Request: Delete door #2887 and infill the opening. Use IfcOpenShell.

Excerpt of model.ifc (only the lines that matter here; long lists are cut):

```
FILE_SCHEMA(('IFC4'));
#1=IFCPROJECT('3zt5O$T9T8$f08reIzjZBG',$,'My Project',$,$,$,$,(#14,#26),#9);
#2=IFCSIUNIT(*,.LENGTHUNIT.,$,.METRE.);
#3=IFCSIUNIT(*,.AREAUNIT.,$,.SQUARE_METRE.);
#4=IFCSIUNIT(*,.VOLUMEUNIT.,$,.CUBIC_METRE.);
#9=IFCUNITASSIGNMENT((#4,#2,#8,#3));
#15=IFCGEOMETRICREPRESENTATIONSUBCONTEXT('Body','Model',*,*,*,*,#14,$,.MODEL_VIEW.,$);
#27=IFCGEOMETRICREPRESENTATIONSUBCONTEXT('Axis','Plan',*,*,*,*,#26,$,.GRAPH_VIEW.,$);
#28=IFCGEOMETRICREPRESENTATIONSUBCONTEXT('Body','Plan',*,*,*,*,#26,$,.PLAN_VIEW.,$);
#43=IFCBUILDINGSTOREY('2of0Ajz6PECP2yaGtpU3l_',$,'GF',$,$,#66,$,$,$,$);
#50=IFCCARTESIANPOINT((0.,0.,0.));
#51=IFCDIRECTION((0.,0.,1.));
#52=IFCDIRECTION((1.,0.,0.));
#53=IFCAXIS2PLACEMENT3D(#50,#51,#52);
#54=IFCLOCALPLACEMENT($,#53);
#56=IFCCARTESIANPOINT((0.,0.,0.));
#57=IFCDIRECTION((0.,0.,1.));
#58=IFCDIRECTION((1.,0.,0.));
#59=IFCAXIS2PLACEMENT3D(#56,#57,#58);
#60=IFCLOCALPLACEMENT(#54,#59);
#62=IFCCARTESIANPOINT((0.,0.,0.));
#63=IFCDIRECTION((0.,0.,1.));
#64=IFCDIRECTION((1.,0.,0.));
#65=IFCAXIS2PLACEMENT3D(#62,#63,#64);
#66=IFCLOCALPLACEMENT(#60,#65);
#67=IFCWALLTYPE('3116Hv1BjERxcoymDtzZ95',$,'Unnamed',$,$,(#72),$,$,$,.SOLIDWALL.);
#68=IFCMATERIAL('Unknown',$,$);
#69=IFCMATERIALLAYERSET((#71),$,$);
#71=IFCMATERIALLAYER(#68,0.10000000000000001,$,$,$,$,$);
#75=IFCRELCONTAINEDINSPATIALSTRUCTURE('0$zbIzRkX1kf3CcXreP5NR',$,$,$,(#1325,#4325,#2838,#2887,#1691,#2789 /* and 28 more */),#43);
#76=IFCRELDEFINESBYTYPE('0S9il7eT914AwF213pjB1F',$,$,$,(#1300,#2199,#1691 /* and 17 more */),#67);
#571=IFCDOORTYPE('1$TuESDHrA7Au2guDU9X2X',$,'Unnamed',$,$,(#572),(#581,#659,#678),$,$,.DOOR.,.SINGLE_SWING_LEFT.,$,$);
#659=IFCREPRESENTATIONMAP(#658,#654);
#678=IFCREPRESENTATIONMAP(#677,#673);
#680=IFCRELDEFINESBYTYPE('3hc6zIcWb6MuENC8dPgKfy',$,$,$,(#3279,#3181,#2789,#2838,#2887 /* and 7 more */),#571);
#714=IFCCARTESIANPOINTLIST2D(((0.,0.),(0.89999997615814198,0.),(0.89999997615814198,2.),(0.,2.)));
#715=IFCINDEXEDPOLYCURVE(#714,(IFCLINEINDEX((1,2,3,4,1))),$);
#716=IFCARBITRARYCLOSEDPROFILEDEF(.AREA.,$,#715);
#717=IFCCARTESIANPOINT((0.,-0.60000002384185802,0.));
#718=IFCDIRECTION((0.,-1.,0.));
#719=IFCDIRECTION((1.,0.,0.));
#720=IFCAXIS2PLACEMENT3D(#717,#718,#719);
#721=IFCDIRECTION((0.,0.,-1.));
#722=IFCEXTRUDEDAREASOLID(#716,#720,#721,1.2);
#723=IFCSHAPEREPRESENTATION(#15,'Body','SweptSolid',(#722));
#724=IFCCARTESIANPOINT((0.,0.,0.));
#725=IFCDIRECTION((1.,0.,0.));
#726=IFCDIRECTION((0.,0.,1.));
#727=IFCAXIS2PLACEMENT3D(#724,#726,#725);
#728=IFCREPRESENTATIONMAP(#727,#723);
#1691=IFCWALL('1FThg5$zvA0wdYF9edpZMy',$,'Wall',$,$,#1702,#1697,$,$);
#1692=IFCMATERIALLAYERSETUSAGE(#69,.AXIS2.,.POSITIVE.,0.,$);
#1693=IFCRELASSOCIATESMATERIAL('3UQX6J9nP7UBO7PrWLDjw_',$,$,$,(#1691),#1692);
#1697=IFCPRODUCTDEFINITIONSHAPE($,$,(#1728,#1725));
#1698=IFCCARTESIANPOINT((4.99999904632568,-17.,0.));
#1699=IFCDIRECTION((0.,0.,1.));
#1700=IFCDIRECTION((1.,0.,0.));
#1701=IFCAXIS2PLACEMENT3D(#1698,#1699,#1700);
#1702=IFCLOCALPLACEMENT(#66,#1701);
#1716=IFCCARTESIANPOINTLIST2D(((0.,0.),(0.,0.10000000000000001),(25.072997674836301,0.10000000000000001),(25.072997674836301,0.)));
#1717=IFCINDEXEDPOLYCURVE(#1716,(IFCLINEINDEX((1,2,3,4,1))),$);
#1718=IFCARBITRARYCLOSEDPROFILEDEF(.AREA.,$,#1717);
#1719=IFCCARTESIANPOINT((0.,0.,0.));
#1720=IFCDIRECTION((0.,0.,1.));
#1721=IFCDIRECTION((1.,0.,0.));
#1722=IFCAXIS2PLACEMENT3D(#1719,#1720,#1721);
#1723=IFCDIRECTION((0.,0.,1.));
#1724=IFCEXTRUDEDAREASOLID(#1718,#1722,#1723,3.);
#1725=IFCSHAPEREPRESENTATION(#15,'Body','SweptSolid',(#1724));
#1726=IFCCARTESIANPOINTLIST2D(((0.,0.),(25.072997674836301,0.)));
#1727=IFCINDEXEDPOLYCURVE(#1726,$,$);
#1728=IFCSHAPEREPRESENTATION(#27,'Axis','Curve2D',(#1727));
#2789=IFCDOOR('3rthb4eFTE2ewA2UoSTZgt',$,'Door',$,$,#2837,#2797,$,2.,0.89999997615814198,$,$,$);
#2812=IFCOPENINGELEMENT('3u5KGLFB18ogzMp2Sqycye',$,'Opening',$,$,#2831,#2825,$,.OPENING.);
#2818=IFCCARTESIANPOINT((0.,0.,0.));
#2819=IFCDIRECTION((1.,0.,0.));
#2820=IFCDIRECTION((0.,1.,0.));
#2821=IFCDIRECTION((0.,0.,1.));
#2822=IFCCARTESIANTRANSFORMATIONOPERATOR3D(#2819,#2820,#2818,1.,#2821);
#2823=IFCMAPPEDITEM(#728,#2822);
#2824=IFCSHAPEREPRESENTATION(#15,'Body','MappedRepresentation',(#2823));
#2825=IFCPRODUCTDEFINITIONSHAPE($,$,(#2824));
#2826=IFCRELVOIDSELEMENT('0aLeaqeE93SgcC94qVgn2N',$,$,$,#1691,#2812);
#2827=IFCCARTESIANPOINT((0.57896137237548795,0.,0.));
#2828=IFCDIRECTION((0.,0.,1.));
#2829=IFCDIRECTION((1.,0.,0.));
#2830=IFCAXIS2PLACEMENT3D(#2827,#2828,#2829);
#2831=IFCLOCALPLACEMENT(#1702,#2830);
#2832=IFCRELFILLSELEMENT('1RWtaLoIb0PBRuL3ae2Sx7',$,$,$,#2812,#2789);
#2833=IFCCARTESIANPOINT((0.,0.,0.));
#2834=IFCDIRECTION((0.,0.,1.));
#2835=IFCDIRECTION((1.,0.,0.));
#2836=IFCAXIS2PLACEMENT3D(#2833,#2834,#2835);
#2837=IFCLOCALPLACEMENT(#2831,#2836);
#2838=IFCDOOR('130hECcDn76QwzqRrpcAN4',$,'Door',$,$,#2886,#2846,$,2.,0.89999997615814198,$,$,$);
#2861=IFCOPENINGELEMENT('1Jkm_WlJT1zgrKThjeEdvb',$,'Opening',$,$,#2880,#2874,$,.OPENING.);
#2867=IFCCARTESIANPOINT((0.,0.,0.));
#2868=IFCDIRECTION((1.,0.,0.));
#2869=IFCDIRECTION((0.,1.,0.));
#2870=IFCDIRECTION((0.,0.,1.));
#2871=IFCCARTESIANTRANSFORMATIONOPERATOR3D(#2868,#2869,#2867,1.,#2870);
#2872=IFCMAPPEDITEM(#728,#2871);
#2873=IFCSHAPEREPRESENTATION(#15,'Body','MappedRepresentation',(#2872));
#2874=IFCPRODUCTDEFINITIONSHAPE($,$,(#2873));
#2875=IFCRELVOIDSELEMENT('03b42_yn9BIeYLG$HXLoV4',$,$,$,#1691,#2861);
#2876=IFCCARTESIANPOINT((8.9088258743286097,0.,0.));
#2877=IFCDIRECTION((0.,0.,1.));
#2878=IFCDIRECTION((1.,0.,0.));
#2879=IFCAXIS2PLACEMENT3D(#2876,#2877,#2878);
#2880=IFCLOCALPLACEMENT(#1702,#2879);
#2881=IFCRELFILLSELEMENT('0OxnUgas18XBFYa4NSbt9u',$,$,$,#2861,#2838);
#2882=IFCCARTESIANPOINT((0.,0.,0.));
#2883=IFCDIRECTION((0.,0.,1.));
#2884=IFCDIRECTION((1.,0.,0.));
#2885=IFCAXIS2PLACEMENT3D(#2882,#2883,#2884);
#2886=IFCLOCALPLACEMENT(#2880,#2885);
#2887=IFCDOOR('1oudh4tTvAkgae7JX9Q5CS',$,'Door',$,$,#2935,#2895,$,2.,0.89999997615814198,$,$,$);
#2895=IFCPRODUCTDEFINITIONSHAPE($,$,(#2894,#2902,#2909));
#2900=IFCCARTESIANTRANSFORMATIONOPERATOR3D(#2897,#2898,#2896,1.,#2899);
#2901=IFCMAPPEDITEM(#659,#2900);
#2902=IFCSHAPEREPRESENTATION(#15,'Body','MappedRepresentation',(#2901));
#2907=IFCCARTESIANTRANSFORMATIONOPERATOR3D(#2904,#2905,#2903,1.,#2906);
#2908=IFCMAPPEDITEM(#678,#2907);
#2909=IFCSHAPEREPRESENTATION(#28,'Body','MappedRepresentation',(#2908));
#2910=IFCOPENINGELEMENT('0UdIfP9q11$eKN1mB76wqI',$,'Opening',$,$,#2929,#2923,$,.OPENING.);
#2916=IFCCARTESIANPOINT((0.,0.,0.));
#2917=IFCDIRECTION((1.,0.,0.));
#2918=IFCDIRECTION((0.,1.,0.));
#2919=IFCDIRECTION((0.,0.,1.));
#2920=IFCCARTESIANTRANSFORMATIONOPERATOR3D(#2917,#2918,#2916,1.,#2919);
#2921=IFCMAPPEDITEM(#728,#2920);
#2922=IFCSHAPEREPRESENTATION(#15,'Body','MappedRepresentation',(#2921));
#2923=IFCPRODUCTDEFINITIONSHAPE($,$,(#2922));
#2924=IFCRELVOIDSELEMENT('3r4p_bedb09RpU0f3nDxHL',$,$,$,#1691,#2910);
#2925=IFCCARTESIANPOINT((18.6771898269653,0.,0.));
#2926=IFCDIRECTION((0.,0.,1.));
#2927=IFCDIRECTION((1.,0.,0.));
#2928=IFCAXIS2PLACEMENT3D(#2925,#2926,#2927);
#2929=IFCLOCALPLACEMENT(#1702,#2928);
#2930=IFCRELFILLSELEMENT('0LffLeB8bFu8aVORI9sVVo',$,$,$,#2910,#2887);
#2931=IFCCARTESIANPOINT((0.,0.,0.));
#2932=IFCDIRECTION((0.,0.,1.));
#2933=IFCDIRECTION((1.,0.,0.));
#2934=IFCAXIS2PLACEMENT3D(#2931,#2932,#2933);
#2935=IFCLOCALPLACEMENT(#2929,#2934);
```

```python
import ifcopenshell
import ifcopenshell.api.feature
import ifcopenshell.api.root
import ifcopenshell.geom
import ifcopenshell.util.shape

model = ifcopenshell.open("model.ifc")
settings = ifcopenshell.geom.settings()


def volume(element):
    """Net volume in cubic metres, openings subtracted."""
    shape = ifcopenshell.geom.create_shape(settings, element)
    return ifcopenshell.util.shape.get_volume(shape.geometry)


door = model.by_guid("1oudh4tTvAkgae7JX9Q5CS")
opening = door.FillsVoids[0].RelatingOpeningElement
wall = opening.VoidsElements[0].RelatingBuildingElement
before = volume(wall)

ifcopenshell.api.root.remove_product(model, product=door)
ifcopenshell.api.feature.remove_feature(model, feature=opening)

after = volume(wall)

print(f"wall volume {before:.3f} -> {after:.3f} m3")

model.write("model-out.ifc")
```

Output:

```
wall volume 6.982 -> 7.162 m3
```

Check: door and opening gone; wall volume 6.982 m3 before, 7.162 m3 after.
